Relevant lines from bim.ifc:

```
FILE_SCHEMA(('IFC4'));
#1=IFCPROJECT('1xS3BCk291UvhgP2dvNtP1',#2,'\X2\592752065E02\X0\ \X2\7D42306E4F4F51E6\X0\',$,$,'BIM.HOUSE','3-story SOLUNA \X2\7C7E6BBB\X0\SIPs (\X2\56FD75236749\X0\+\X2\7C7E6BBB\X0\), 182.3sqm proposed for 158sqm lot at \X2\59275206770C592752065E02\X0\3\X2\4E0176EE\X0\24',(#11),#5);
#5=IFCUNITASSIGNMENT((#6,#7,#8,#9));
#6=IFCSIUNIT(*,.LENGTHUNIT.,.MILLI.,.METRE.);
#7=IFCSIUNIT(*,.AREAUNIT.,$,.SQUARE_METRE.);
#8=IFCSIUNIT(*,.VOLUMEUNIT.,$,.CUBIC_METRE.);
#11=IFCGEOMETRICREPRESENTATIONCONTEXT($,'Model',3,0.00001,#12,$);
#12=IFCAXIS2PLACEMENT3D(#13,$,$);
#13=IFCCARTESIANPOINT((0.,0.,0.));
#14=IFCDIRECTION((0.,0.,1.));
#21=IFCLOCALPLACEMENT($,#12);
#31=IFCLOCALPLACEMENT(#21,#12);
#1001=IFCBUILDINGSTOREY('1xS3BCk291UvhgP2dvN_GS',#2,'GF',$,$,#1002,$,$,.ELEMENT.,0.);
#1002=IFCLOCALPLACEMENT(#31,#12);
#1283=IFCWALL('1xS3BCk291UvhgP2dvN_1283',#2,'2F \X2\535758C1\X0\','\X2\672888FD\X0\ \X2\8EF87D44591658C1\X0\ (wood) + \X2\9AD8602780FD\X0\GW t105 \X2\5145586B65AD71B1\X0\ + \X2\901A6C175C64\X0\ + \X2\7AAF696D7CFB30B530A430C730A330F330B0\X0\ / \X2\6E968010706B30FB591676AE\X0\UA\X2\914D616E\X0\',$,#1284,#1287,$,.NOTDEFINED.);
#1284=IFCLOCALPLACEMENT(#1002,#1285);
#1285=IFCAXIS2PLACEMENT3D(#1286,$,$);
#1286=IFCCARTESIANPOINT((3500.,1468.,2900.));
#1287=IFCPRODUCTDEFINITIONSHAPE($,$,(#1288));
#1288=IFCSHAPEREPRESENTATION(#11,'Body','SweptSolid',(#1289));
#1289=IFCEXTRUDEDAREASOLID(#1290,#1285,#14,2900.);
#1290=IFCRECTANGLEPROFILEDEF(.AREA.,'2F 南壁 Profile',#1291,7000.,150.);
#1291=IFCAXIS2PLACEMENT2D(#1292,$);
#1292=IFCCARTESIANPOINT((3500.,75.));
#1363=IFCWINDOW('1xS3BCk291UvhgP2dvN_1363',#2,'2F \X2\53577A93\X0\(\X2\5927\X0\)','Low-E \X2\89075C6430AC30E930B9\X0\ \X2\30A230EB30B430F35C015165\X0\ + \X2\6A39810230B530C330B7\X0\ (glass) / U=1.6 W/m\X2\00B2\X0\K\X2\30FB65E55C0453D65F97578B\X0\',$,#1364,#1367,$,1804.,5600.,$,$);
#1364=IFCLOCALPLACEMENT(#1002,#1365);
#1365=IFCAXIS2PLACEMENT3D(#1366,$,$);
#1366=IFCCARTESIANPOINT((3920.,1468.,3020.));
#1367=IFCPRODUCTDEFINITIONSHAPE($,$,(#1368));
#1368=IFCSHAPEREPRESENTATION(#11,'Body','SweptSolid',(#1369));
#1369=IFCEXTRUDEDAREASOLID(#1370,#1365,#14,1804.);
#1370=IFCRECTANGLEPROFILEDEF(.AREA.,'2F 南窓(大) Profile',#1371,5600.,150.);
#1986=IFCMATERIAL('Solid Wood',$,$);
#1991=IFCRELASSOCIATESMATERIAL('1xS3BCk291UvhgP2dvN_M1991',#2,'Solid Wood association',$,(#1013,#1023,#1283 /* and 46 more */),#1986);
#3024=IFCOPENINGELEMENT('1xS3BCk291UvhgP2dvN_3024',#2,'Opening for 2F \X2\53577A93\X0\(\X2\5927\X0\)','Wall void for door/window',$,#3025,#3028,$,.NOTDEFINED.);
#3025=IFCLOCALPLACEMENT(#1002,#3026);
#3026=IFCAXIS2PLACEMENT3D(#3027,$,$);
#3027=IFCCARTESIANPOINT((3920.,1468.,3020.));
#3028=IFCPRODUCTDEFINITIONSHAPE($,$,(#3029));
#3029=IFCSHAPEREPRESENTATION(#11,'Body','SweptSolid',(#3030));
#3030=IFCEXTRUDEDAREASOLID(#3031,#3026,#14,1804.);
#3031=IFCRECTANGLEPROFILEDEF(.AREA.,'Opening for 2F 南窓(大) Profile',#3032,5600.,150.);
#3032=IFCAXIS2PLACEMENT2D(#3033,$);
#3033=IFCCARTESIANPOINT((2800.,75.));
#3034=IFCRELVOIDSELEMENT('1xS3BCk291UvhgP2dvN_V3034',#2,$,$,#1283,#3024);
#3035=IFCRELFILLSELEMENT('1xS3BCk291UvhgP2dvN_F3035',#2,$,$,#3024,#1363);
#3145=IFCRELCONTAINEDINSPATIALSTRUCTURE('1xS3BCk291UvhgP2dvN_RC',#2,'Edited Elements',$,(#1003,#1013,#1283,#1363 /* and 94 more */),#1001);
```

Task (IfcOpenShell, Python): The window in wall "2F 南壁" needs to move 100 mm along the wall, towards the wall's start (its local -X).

```python
import ifcopenshell
import ifcopenshell.api.geometry
import ifcopenshell.util.placement

model = ifcopenshell.open("bim.ifc")

window = model.by_id(1363)
opening = window.FillsVoids[0].RelatingOpeningElement
wall = opening.VoidsElements[0].RelatingBuildingElement

wall_matrix = ifcopenshell.util.placement.get_local_placement(wall.ObjectPlacement)
shift = wall_matrix[:3, 0] * -100.0
before = ifcopenshell.util.placement.get_local_placement(window.ObjectPlacement)[:3, 3].copy()

# The window is not placed relative to its opening, so move both.
for product in (opening, window):
    matrix = ifcopenshell.util.placement.get_local_placement(product.ObjectPlacement)
    matrix[:3, 3] += shift
    ifcopenshell.api.geometry.edit_object_placement(model, product=product, matrix=matrix, is_si=False)

after = ifcopenshell.util.placement.get_local_placement(window.ObjectPlacement)[:3, 3]
print("window moved by", (after - before).round(3) + 0.0)

model.write("bim_v2.ifc")
```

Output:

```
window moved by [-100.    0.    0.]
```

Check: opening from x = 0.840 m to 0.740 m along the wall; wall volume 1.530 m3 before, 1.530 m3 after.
